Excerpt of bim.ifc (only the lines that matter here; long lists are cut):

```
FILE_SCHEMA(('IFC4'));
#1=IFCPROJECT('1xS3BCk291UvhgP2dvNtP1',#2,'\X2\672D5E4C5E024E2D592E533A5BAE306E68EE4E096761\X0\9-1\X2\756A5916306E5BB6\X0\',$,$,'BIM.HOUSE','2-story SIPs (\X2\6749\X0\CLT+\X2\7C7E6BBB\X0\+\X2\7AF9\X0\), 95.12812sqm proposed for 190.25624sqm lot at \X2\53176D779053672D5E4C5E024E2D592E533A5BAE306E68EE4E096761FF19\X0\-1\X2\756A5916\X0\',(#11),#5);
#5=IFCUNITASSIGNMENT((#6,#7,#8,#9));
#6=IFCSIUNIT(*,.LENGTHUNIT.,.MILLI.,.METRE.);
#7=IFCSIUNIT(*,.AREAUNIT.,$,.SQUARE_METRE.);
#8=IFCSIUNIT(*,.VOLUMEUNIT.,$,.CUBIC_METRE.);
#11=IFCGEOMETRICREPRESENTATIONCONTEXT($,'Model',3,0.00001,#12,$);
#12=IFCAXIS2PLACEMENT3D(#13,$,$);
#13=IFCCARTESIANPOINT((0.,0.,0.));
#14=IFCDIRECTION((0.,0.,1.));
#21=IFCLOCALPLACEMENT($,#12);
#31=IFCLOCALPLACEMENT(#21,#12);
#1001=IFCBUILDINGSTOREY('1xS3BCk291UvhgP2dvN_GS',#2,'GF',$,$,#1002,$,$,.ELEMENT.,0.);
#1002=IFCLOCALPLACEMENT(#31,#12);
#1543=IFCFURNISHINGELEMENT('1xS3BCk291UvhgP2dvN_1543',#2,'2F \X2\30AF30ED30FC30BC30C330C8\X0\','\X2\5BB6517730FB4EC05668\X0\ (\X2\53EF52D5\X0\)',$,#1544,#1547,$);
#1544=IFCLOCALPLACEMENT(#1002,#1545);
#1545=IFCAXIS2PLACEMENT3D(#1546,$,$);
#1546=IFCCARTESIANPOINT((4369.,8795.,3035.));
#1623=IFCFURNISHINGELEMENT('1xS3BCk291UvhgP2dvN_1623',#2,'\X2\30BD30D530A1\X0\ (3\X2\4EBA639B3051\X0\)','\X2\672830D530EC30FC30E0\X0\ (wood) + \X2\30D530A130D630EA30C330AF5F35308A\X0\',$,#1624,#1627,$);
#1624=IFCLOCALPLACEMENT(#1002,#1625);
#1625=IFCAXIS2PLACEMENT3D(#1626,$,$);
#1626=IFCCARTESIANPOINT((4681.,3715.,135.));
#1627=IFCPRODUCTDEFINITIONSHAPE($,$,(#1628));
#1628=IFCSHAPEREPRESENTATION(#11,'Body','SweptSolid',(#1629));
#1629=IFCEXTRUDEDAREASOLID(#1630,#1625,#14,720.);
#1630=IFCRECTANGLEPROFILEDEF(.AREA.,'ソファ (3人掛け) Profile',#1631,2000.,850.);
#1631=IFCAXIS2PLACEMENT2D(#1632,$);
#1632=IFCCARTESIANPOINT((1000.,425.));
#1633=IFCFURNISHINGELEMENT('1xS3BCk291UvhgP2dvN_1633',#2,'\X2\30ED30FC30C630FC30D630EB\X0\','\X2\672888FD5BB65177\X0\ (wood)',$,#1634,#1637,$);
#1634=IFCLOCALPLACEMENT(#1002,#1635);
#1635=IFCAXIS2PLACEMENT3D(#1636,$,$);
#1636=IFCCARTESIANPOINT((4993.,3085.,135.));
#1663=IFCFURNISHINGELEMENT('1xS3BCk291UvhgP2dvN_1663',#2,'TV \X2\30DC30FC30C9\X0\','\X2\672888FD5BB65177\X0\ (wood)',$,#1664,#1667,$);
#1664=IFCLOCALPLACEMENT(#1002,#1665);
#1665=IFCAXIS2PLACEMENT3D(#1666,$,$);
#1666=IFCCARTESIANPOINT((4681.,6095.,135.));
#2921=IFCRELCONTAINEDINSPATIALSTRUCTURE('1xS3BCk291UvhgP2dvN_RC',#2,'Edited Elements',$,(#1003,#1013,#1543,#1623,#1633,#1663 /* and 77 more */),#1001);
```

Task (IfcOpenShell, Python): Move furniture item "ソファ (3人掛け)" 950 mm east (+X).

```python
import ifcopenshell
import ifcopenshell.api.geometry
import ifcopenshell.util.placement

model = ifcopenshell.open("bim.ifc")

item = model.by_guid("1xS3BCk291UvhgP2dvN_1623")
matrix = ifcopenshell.util.placement.get_local_placement(item.ObjectPlacement)
matrix[0, 3] += 950.0
ifcopenshell.api.geometry.edit_object_placement(model, product=item, matrix=matrix, is_si=False)

print(ifcopenshell.util.placement.get_local_placement(item.ObjectPlacement).round(3) + 0.0)

model.write("bim_v2.ifc")
```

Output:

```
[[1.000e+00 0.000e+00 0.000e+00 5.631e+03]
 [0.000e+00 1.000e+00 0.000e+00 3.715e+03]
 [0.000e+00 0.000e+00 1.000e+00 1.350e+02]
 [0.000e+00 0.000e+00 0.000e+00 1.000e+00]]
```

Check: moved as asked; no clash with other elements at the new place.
